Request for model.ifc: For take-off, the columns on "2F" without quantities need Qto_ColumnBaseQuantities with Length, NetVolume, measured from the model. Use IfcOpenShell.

First a look at what the model holds.

```python
import ifcopenshell
import ifcopenshell.util.element
import ifcopenshell.util.unit

model = ifcopenshell.open("model.ifc")
print(model.schema)
for unit_type in ("LENGTHUNIT", "AREAUNIT", "VOLUMEUNIT"):
    print(unit_type, ifcopenshell.util.unit.calculate_unit_scale(model, unit_type))
storey = next(s for s in model.by_type("IfcBuildingStorey") if s.Name == "2F")
columns = [e for e in ifcopenshell.util.element.get_decomposition(storey) if e.is_a("IfcColumn")]
for e in sorted(columns, key=lambda e: e.id()):
    print(e.id(), e.is_a(), e.Name, list(ifcopenshell.util.element.get_psets(e, qtos_only=True)), sep=" | ")
```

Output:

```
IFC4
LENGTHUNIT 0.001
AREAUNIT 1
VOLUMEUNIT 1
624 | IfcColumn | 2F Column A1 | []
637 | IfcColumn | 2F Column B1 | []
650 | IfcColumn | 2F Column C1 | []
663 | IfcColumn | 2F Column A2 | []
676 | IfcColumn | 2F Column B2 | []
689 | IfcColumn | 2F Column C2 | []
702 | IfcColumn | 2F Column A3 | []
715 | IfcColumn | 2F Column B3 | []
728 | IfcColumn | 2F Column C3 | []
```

```python
import ifcopenshell
import ifcopenshell.api.pset
import ifcopenshell.geom
import ifcopenshell.util.element
import ifcopenshell.util.shape
import ifcopenshell.util.unit

model = ifcopenshell.open("model.ifc")
unit_scale = ifcopenshell.util.unit.calculate_unit_scale(model)
volume_scale = ifcopenshell.util.unit.calculate_unit_scale(model, "VOLUMEUNIT")
settings = ifcopenshell.geom.settings()

storey = next(s for s in model.by_type("IfcBuildingStorey") if s.Name == "2F")
columns = [e for e in ifcopenshell.util.element.get_decomposition(storey) if e.is_a("IfcColumn")]

for e in sorted(columns, key=lambda e: e.id()):
    if ifcopenshell.util.element.get_psets(e, qtos_only=True, should_inherit=False):
        continue
    # Geometry comes back in metres, in the element's own axes.
    shape = ifcopenshell.geom.create_shape(settings, e)
    values = {
        "Length": ifcopenshell.util.shape.get_z(shape.geometry) / unit_scale,
        "NetVolume": ifcopenshell.util.shape.get_volume(shape.geometry) / volume_scale,
    }
    qto = ifcopenshell.api.pset.add_qto(model, product=e, name="Qto_ColumnBaseQuantities")
    ifcopenshell.api.pset.edit_qto(model, qto=qto, properties=values)
    print(e.id(), {k: round(v, 3) for k, v in values.items()})

model.write("model_rev.ifc")
```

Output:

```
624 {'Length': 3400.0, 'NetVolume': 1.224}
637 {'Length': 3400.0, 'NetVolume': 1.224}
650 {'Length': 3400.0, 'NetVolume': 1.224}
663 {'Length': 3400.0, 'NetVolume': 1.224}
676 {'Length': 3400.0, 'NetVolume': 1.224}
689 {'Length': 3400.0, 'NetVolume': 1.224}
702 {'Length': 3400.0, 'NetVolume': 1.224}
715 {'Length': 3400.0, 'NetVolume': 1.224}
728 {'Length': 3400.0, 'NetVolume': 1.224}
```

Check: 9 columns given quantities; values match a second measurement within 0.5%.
